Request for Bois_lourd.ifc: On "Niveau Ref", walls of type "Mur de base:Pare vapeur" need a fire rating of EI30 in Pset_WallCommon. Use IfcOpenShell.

First a look at what the model holds.

```python
import ifcopenshell
import ifcopenshell.util.element

model = ifcopenshell.open("Bois_lourd.ifc")
print(model.schema)
storey = next(s for s in model.by_type("IfcBuildingStorey") if s.Name == "Niveau Ref")
walls = [e for e in ifcopenshell.util.element.get_decomposition(storey) if e.is_a("IfcWall")]
seen = {}
for e in walls:
    element_type = ifcopenshell.util.element.get_type(e)
    key = (element_type.Name if element_type != e and element_type else None, ifcopenshell.util.element.get_pset(e, "Pset_WallCommon", "FireRating"))
    seen[key] = seen.get(key, 0) + 1
for (name, value), count in sorted(seen.items(), key=str):
    print(count, "x", name, "|", value)
```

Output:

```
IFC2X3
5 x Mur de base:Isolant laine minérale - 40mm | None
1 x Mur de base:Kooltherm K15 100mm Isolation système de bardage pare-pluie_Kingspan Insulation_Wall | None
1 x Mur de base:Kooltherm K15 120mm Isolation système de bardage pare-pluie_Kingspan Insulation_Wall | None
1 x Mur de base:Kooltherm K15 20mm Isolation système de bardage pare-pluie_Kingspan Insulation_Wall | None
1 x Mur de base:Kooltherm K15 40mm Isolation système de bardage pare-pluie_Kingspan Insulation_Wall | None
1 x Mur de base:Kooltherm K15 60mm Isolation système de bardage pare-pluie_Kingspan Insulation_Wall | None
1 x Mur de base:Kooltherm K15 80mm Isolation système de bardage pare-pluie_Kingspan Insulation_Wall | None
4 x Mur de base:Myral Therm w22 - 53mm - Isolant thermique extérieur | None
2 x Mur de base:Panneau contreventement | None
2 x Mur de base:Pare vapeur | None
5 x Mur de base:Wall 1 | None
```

```python
import ifcopenshell
import ifcopenshell.api.pset
import ifcopenshell.util.element

model = ifcopenshell.open("Bois_lourd.ifc")

storey = next(s for s in model.by_type("IfcBuildingStorey") if s.Name == "Niveau Ref")
walls = [e for e in ifcopenshell.util.element.get_decomposition(storey) if e.is_a("IfcWall")]

count = 0
for e in walls:
    element_type = ifcopenshell.util.element.get_type(e)
    if element_type in (None, e) or element_type.Name != "Mur de base:Pare vapeur":
        continue
    # add_pset returns the element's existing set when there is one.
    pset = ifcopenshell.api.pset.add_pset(model, product=e, name="Pset_WallCommon")
    ifcopenshell.api.pset.edit_pset(model, pset=pset, properties={"FireRating": "EI30"})
    count += 1

print(count, "walls updated")

model.write("Bois_lourd_edited.ifc")
```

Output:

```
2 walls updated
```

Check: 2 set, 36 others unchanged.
